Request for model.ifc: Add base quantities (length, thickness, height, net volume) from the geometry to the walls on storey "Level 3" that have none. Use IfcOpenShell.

First a look at what the model holds.

```python
import ifcopenshell
import ifcopenshell.util.element
import ifcopenshell.util.unit

model = ifcopenshell.open("model.ifc")
print(model.schema)
for unit_type in ("LENGTHUNIT", "AREAUNIT", "VOLUMEUNIT"):
    print(unit_type, ifcopenshell.util.unit.calculate_unit_scale(model, unit_type))
storey = next(s for s in model.by_type("IfcBuildingStorey") if s.Name == "Level 3")
walls = [e for e in ifcopenshell.util.element.get_decomposition(storey) if e.is_a("IfcWall")]
for e in sorted(walls, key=lambda e: e.id()):
    print(e.id(), e.is_a(), e.Name, list(ifcopenshell.util.element.get_psets(e, qtos_only=True)), sep=" | ")
```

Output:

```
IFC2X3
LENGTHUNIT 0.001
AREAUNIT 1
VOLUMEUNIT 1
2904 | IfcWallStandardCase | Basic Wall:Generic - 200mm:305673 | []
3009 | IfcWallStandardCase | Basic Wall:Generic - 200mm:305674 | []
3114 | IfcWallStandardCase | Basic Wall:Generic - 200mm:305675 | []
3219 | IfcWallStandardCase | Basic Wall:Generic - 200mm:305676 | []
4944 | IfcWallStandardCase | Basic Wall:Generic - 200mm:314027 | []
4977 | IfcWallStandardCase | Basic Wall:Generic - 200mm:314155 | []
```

```python
import ifcopenshell
import ifcopenshell.api.pset
import ifcopenshell.geom
import ifcopenshell.util.element
import ifcopenshell.util.shape
import ifcopenshell.util.unit

model = ifcopenshell.open("model.ifc")
unit_scale = ifcopenshell.util.unit.calculate_unit_scale(model)
volume_scale = ifcopenshell.util.unit.calculate_unit_scale(model, "VOLUMEUNIT")
settings = ifcopenshell.geom.settings()

storey = next(s for s in model.by_type("IfcBuildingStorey") if s.Name == "Level 3")
walls = [e for e in ifcopenshell.util.element.get_decomposition(storey) if e.is_a("IfcWall")]

for e in sorted(walls, key=lambda e: e.id()):
    if ifcopenshell.util.element.get_psets(e, qtos_only=True, should_inherit=False):
        continue
    # Geometry comes back in metres, in the element's own axes.
    shape = ifcopenshell.geom.create_shape(settings, e)
    values = {
        "Length": ifcopenshell.util.shape.get_x(shape.geometry) / unit_scale,
        "Width": ifcopenshell.util.shape.get_y(shape.geometry) / unit_scale,
        "Height": ifcopenshell.util.shape.get_z(shape.geometry) / unit_scale,
        "NetVolume": ifcopenshell.util.shape.get_volume(shape.geometry) / volume_scale,
    }
    qto = ifcopenshell.api.pset.add_qto(model, product=e, name="BaseQuantities")
    ifcopenshell.api.pset.edit_qto(model, qto=qto, properties=values)
    print(e.id(), {k: round(v, 3) for k, v in values.items()})

model.write("model-out.ifc")
```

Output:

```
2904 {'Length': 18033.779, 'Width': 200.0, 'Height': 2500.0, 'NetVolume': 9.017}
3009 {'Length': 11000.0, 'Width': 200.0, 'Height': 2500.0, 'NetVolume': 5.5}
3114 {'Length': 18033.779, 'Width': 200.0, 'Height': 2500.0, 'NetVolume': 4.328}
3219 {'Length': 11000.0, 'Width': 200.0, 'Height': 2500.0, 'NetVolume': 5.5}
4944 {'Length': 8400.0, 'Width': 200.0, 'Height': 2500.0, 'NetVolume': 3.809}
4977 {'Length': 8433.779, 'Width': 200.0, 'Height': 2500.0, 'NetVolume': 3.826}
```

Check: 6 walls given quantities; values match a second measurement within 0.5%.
